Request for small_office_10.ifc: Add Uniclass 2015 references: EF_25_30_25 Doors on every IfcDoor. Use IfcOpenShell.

First a look at what the model holds.

```python
import ifcopenshell

model = ifcopenshell.open("small_office_10.ifc")
print(model.schema)
print("classifications:", [c.Name for c in model.by_type("IfcClassification")])
for ifc_class in ("IfcDoor", "IfcRoof", "IfcStair", "IfcWall", "IfcWindow"):
    print(ifc_class, len(model.by_type(ifc_class)))
```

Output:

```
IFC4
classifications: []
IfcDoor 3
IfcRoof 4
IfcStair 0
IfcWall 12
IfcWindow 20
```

```python
import ifcopenshell
import ifcopenshell.api.classification

model = ifcopenshell.open("small_office_10.ifc")

system = ifcopenshell.api.classification.add_classification(model, classification="Uniclass 2015")

codes = {
    "IfcDoor": ("EF_25_30_25", "Doors"),
}
for ifc_class, (code, name) in codes.items():
    products = model.by_type(ifc_class)
    ifcopenshell.api.classification.add_reference(
        model, products=products, classification=system, identification=code, name=name
    )
    print(code, len(products))

model.write("small_office_10_v2.ifc")
```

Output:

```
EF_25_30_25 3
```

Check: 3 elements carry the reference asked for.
